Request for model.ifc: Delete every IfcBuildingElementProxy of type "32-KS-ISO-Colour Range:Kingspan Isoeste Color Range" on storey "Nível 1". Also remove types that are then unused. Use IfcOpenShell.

First a look at what the model holds.

```python
import ifcopenshell
import ifcopenshell.util.element

model = ifcopenshell.open("model.ifc")
print(model.schema)
storey = next(s for s in model.by_type("IfcBuildingStorey") if s.Name == "Nível 1")
proxies = [e for e in ifcopenshell.util.element.get_decomposition(storey) if e.is_a("IfcBuildingElementProxy")]
seen = {}
for e in proxies:
    element_type = ifcopenshell.util.element.get_type(e)
    name = element_type.Name if element_type not in (None, e) else None
    seen[name] = seen.get(name, 0) + 1
for name, count in sorted(seen.items(), key=str):
    print(count, "x", name)
```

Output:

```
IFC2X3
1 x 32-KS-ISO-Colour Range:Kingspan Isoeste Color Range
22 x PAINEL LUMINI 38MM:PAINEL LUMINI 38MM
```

```python
import ifcopenshell
import ifcopenshell.api.root
import ifcopenshell.util.element

model = ifcopenshell.open("model.ifc")

storey = next(s for s in model.by_type("IfcBuildingStorey") if s.Name == "Nível 1")
proxies = [e for e in ifcopenshell.util.element.get_decomposition(storey) if e.is_a("IfcBuildingElementProxy")]
targets = [e for e in proxies if (t := ifcopenshell.util.element.get_type(e)) not in (None, e) and t.Name == "32-KS-ISO-Colour Range:Kingspan Isoeste Color Range"]
types = {ifcopenshell.util.element.get_type(e) for e in targets} - {None, *targets}

for e in targets:
    ifcopenshell.api.root.remove_product(model, product=e)
print(len(targets), "removed")

unused = [t for t in types if not ifcopenshell.util.element.get_types(t)]
for t in unused:
    ifcopenshell.api.root.remove_product(model, product=t)
print(len(unused), "unused types removed")

model.write("model_edited.ifc")
```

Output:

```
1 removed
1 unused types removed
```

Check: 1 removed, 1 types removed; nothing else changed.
